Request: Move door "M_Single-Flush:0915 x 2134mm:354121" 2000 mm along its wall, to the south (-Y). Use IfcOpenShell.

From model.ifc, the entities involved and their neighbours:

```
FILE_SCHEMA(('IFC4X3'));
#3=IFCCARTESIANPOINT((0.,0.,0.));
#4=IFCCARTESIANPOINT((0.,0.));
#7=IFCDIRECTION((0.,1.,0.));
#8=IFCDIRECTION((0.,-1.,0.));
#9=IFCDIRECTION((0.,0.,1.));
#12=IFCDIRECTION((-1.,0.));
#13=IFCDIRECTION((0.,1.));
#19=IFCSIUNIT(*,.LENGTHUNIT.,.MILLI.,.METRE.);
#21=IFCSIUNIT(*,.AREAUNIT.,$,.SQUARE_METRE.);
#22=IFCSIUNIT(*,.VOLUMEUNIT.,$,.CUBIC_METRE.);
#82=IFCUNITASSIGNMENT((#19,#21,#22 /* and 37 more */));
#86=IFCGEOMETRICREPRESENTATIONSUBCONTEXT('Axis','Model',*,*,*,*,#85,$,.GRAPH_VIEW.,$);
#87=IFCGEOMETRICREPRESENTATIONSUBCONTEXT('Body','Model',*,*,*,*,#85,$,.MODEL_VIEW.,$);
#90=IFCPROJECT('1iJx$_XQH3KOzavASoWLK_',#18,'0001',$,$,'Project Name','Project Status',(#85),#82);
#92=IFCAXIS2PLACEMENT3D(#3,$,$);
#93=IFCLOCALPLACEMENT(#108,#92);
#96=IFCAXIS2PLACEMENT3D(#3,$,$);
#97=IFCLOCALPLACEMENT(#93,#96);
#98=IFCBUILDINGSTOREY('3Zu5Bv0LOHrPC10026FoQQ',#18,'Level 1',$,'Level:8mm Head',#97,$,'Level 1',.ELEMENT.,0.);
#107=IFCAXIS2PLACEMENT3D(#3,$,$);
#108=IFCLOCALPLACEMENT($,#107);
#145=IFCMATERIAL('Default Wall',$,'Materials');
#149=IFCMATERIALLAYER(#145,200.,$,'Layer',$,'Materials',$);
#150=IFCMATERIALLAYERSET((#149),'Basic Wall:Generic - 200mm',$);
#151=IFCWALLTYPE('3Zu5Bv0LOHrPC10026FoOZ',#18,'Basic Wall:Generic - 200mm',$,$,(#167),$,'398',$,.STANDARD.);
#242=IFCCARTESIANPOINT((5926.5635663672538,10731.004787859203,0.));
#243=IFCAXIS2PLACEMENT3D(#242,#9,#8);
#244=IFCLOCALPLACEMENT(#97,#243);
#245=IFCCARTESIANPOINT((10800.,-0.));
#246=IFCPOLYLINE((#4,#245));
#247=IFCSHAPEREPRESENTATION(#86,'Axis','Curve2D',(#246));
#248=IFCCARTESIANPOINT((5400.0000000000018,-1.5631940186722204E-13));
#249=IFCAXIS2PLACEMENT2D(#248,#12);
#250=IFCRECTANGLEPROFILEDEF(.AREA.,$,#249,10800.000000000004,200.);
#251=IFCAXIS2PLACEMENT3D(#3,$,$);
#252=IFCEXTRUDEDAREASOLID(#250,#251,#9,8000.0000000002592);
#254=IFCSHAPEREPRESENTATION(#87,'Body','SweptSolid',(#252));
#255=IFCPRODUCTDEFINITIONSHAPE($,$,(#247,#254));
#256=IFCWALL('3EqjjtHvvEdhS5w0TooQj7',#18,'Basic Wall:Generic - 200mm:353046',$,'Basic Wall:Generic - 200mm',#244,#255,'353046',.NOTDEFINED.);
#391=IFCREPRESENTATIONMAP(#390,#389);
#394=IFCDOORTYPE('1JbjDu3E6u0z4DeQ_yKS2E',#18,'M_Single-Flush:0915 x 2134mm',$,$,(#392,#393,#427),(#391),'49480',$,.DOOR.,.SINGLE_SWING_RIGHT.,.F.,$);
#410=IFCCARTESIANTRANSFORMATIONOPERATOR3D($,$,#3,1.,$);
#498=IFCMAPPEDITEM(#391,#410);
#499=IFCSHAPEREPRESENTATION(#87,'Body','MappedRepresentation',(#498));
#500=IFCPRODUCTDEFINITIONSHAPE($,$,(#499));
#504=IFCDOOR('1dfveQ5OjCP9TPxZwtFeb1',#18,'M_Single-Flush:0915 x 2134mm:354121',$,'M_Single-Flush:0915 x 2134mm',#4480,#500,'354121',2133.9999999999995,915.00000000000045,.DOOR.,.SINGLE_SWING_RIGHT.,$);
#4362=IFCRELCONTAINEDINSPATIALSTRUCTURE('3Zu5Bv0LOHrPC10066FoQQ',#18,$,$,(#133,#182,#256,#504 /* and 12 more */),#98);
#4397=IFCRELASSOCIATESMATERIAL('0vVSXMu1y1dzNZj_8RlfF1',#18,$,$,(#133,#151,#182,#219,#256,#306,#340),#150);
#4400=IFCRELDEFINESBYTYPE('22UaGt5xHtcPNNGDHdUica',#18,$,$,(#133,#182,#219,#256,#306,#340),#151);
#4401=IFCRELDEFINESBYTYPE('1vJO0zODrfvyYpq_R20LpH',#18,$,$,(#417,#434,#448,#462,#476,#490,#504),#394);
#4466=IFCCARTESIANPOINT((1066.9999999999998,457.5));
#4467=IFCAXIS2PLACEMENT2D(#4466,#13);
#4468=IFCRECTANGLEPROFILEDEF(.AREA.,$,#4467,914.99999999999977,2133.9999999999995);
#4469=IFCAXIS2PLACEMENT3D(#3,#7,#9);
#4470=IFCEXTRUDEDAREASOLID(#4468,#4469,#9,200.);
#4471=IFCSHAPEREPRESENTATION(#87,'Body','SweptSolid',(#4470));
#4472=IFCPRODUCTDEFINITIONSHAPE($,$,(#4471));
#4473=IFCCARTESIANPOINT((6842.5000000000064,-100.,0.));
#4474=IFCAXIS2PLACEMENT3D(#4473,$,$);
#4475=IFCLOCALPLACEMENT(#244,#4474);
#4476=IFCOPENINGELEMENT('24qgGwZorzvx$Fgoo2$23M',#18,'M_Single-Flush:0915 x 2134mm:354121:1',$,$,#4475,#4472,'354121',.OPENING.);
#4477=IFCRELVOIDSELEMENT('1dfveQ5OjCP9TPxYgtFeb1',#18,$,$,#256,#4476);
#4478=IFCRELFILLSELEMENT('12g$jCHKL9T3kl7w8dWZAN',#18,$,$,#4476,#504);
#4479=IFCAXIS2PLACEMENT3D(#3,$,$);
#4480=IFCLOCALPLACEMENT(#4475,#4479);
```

```python
import ifcopenshell
import ifcopenshell.api.geometry
import ifcopenshell.util.placement

model = ifcopenshell.open("model.ifc")

door = model.by_guid("1dfveQ5OjCP9TPxZwtFeb1")
opening = door.FillsVoids[0].RelatingOpeningElement
wall = opening.VoidsElements[0].RelatingBuildingElement

wall_matrix = ifcopenshell.util.placement.get_local_placement(wall.ObjectPlacement)
shift = wall_matrix[:3, 0] * 2000.0
before = ifcopenshell.util.placement.get_local_placement(door.ObjectPlacement)[:3, 3].copy()

# The door is placed relative to its opening, so it follows when the opening moves.
matrix = ifcopenshell.util.placement.get_local_placement(opening.ObjectPlacement)
matrix[:3, 3] += shift
ifcopenshell.api.geometry.edit_object_placement(
    model, product=opening, matrix=matrix, is_si=False, should_transform_children=True
)

after = ifcopenshell.util.placement.get_local_placement(door.ObjectPlacement)[:3, 3]
print("door moved by", (after - before).round(3) + 0.0)

model.write("model_edited.ifc")
```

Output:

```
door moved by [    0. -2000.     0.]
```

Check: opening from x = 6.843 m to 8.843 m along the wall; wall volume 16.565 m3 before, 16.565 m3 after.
